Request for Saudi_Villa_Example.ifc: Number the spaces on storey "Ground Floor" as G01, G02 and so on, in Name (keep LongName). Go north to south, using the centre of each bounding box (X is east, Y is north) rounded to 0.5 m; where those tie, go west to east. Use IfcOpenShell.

First a look at what the model holds.

```python
import ifcopenshell
import ifcopenshell.util.element
import ifcopenshell.util.placement

model = ifcopenshell.open("Saudi_Villa_Example.ifc")
print(model.schema)
storey = next(s for s in model.by_type("IfcBuildingStorey") if s.Name == "Ground Floor")
spaces = [e for e in ifcopenshell.util.element.get_decomposition(storey) if e.is_a("IfcSpace")]
for e in sorted(spaces, key=lambda e: e.id()):
    origin = ifcopenshell.util.placement.get_local_placement(e.ObjectPlacement)[:3, 3]
    print(e.id(), e.Name, e.LongName, origin.round(2) + 0.0, sep=" | ")
```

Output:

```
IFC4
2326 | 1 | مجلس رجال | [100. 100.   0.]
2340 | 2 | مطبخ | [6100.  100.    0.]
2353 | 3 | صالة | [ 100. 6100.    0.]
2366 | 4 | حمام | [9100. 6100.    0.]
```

```python
import ifcopenshell
import ifcopenshell.geom
import ifcopenshell.util.element
import ifcopenshell.util.shape

model = ifcopenshell.open("Saudi_Villa_Example.ifc")
settings = ifcopenshell.geom.settings()
settings.set("use-world-coords", True)


def centre(element):
    shape = ifcopenshell.geom.create_shape(settings, element)
    return ifcopenshell.util.shape.get_bbox_centroid(shape.geometry)


storey = next(s for s in model.by_type("IfcBuildingStorey") if s.Name == "Ground Floor")
spaces = [e for e in ifcopenshell.util.element.get_decomposition(storey) if e.is_a("IfcSpace")]

# Insertion points can sit at a corner or the storey origin, so sort by the geometry (in metres).
centres = {e: centre(e) for e in spaces}
spaces.sort(key=lambda e: (-round(centres[e][1] / 0.5), centres[e][0]))

for i, e in enumerate(spaces, start=1):
    number = f"G{i:02d}"
    e.Name = number
    print(e.id(), number)

model.write("Saudi_Villa_Example_edited.ifc")
```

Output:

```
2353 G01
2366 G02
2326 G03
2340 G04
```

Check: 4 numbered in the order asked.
